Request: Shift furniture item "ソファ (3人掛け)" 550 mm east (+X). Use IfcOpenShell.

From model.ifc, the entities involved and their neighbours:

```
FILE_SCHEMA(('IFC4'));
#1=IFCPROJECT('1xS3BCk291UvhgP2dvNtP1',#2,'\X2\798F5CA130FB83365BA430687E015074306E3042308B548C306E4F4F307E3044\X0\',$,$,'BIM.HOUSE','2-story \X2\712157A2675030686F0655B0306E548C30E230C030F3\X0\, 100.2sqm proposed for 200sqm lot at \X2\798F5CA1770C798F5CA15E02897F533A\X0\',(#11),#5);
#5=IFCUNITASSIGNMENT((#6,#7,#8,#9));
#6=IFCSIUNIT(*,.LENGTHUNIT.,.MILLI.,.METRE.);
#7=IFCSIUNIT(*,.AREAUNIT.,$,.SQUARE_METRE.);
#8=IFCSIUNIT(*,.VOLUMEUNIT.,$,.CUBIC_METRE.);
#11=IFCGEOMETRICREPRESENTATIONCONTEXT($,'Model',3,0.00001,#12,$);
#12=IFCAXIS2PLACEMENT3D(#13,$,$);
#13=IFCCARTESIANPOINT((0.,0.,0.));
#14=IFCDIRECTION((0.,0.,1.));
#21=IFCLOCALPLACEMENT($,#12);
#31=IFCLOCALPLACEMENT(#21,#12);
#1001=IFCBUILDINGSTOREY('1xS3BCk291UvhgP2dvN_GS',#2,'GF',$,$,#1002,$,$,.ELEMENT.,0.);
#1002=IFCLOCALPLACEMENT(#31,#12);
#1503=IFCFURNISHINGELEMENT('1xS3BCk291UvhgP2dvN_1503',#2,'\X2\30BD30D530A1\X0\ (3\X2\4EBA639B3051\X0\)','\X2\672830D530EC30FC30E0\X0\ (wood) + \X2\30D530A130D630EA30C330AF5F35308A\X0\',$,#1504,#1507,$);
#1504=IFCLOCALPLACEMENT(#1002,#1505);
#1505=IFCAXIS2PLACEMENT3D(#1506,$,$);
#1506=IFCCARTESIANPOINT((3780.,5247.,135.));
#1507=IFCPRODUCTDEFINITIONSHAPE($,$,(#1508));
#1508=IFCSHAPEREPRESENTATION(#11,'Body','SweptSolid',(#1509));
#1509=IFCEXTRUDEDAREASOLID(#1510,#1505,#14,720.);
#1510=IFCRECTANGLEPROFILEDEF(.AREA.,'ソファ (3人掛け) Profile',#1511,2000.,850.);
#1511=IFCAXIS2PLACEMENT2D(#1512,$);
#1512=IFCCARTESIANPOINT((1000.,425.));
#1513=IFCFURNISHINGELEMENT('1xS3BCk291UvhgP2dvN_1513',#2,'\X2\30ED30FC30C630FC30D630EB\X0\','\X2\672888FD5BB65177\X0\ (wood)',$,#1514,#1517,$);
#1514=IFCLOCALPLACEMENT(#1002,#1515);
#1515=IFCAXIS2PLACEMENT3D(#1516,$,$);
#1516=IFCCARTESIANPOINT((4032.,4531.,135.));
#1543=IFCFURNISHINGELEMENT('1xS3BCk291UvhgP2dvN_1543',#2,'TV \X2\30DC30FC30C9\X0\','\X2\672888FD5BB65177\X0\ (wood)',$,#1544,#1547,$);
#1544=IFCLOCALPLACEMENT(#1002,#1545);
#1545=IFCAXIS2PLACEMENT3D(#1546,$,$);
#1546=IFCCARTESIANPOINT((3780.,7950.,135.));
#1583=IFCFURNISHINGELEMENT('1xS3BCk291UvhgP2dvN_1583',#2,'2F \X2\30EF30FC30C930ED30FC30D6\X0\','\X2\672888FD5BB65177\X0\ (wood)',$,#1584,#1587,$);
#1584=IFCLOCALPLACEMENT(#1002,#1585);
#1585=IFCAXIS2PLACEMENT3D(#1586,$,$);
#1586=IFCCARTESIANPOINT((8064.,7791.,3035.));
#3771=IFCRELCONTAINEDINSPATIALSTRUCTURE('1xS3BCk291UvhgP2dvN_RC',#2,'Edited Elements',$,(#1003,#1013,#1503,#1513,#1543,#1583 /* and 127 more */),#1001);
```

```python
import ifcopenshell
import ifcopenshell.api.geometry
import ifcopenshell.util.placement
import ifcopenshell.util.unit

model = ifcopenshell.open("model.ifc")
unit_scale = ifcopenshell.util.unit.calculate_unit_scale(model)

item = model.by_guid("1xS3BCk291UvhgP2dvN_1503")
matrix = ifcopenshell.util.placement.get_local_placement(item.ObjectPlacement)
matrix[0, 3] += 0.55 / unit_scale
ifcopenshell.api.geometry.edit_object_placement(model, product=item, matrix=matrix, is_si=False)

print(ifcopenshell.util.placement.get_local_placement(item.ObjectPlacement).round(3) + 0.0)

model.write("model_updated.ifc")
```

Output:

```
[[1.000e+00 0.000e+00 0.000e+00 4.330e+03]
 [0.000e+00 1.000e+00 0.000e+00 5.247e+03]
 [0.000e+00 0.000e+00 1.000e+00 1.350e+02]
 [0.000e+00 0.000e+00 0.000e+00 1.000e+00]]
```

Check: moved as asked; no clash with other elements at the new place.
